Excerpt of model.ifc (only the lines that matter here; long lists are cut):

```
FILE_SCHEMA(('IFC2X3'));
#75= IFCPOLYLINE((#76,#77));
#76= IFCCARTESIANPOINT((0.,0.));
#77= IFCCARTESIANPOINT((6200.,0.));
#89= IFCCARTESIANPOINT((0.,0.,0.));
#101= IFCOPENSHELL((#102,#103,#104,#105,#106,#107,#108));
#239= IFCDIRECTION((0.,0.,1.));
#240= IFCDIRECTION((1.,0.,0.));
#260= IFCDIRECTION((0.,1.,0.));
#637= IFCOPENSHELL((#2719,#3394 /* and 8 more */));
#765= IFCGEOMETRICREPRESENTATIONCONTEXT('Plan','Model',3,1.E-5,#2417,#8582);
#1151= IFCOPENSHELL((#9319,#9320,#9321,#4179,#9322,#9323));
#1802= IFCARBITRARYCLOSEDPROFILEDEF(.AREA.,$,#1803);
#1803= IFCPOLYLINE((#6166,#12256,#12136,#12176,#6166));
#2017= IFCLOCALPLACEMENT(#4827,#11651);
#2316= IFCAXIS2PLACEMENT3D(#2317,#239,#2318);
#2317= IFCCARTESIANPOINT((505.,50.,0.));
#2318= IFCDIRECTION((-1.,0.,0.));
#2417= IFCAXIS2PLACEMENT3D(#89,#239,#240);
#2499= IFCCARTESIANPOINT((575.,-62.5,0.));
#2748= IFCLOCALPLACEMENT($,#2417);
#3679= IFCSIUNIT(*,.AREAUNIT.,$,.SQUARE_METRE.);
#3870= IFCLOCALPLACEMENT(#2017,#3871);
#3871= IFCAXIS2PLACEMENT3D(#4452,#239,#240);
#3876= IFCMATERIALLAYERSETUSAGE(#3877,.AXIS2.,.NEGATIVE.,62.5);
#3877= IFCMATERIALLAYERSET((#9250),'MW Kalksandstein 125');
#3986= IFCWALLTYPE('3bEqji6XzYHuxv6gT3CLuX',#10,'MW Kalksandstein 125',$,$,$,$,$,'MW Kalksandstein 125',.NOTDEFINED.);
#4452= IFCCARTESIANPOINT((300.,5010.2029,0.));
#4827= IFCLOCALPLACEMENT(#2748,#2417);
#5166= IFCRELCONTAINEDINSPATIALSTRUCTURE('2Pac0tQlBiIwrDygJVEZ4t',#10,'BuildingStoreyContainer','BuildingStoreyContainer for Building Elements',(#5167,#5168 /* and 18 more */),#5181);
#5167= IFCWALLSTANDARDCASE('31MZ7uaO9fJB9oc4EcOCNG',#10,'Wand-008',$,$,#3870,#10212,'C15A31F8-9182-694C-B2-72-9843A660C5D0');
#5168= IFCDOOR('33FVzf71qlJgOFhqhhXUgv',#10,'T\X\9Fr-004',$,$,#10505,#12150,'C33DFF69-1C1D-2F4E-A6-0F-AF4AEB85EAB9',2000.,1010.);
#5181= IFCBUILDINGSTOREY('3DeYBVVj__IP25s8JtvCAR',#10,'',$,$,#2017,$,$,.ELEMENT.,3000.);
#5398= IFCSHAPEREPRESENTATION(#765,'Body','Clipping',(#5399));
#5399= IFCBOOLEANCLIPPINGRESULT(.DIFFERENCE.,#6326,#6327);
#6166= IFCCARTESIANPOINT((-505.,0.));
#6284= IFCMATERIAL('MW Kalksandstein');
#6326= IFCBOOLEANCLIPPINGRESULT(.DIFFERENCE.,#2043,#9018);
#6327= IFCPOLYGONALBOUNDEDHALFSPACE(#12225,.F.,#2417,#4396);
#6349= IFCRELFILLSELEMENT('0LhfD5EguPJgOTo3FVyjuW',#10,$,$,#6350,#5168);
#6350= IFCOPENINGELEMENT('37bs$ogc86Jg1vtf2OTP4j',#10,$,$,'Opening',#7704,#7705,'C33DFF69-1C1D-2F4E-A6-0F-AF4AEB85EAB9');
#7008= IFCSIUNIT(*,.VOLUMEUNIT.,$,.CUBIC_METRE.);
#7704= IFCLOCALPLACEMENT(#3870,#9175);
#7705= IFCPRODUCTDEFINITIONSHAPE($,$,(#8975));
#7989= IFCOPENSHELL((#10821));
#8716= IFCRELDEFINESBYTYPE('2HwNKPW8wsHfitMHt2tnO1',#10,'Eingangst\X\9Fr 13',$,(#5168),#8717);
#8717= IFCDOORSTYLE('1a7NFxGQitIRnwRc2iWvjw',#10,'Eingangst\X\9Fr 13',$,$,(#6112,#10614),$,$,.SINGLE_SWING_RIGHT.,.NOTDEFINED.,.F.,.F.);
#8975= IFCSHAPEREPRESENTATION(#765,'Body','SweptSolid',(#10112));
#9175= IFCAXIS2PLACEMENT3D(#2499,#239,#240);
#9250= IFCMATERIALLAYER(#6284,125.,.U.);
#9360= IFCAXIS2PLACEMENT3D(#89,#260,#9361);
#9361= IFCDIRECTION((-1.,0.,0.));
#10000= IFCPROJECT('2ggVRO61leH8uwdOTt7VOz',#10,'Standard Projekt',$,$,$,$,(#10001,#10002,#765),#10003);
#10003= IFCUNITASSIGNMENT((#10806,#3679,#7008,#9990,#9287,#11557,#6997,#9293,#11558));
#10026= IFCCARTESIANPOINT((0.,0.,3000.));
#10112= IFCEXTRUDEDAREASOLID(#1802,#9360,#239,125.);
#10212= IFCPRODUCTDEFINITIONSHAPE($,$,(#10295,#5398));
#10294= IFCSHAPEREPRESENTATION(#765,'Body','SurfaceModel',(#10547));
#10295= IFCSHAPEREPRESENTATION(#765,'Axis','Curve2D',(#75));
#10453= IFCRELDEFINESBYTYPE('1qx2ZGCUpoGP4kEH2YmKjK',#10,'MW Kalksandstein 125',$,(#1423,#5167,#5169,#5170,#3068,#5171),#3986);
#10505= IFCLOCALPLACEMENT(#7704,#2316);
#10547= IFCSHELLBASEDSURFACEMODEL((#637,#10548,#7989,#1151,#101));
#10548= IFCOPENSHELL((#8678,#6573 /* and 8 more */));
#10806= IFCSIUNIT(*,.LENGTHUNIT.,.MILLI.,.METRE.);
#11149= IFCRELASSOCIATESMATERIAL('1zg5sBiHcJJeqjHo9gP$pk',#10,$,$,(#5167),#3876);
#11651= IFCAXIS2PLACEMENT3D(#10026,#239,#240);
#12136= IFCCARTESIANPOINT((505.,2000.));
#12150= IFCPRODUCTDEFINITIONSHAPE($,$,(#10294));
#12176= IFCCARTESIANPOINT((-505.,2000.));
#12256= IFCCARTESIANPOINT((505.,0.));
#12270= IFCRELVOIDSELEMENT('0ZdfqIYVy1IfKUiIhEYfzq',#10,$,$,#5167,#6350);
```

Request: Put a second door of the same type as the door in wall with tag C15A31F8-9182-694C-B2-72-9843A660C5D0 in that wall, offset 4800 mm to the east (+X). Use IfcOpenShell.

```python
import ifcopenshell
import ifcopenshell.api.feature
import ifcopenshell.api.geometry
import ifcopenshell.api.root
import ifcopenshell.geom
import ifcopenshell.util.element
import ifcopenshell.util.placement
import ifcopenshell.util.shape
import ifcopenshell.util.unit

model = ifcopenshell.open("model.ifc")
unit_scale = ifcopenshell.util.unit.calculate_unit_scale(model)
settings = ifcopenshell.geom.settings()


def volume(element):
    """Net volume in cubic metres, openings subtracted."""
    shape = ifcopenshell.geom.create_shape(settings, element)
    return ifcopenshell.util.shape.get_volume(shape.geometry)


door = model.by_guid("33FVzf71qlJgOFhqhhXUgv")
opening = door.FillsVoids[0].RelatingOpeningElement
wall = opening.VoidsElements[0].RelatingBuildingElement
before = volume(wall)
shift = ifcopenshell.util.placement.get_local_placement(wall.ObjectPlacement)[:3, 0] * 4.8 / unit_scale

# copy_class copies the void relationship, type, container and properties, but no geometry.
new_opening = ifcopenshell.api.root.copy_class(model, product=opening)
new_opening.Representation = ifcopenshell.util.element.copy_deep(
    model, opening.Representation, exclude=["IfcGeometricRepresentationContext", "IfcRepresentationMap"]
)
new_opening.Tag = None
new_door = ifcopenshell.api.root.copy_class(model, product=door)
new_door.Representation = ifcopenshell.util.element.copy_deep(
    model, door.Representation, exclude=["IfcGeometricRepresentationContext", "IfcRepresentationMap"]
)
new_door.Tag = None
fills = ifcopenshell.api.feature.add_filling(model, opening=new_opening, element=new_door)
fills.OwnerHistory = new_door.OwnerHistory  # required in IFC2X3

for old, new in ((opening, new_opening), (door, new_door)):
    matrix = ifcopenshell.util.placement.get_local_placement(old.ObjectPlacement)
    matrix[:3, 3] += shift
    ifcopenshell.api.geometry.edit_object_placement(model, product=new, matrix=matrix, is_si=False)

after = volume(wall)

print(f"wall volume {before:.3f} -> {after:.3f} m3")

model.write("model_edited.ifc")
```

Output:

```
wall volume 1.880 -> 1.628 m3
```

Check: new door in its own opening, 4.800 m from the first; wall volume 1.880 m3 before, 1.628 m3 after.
